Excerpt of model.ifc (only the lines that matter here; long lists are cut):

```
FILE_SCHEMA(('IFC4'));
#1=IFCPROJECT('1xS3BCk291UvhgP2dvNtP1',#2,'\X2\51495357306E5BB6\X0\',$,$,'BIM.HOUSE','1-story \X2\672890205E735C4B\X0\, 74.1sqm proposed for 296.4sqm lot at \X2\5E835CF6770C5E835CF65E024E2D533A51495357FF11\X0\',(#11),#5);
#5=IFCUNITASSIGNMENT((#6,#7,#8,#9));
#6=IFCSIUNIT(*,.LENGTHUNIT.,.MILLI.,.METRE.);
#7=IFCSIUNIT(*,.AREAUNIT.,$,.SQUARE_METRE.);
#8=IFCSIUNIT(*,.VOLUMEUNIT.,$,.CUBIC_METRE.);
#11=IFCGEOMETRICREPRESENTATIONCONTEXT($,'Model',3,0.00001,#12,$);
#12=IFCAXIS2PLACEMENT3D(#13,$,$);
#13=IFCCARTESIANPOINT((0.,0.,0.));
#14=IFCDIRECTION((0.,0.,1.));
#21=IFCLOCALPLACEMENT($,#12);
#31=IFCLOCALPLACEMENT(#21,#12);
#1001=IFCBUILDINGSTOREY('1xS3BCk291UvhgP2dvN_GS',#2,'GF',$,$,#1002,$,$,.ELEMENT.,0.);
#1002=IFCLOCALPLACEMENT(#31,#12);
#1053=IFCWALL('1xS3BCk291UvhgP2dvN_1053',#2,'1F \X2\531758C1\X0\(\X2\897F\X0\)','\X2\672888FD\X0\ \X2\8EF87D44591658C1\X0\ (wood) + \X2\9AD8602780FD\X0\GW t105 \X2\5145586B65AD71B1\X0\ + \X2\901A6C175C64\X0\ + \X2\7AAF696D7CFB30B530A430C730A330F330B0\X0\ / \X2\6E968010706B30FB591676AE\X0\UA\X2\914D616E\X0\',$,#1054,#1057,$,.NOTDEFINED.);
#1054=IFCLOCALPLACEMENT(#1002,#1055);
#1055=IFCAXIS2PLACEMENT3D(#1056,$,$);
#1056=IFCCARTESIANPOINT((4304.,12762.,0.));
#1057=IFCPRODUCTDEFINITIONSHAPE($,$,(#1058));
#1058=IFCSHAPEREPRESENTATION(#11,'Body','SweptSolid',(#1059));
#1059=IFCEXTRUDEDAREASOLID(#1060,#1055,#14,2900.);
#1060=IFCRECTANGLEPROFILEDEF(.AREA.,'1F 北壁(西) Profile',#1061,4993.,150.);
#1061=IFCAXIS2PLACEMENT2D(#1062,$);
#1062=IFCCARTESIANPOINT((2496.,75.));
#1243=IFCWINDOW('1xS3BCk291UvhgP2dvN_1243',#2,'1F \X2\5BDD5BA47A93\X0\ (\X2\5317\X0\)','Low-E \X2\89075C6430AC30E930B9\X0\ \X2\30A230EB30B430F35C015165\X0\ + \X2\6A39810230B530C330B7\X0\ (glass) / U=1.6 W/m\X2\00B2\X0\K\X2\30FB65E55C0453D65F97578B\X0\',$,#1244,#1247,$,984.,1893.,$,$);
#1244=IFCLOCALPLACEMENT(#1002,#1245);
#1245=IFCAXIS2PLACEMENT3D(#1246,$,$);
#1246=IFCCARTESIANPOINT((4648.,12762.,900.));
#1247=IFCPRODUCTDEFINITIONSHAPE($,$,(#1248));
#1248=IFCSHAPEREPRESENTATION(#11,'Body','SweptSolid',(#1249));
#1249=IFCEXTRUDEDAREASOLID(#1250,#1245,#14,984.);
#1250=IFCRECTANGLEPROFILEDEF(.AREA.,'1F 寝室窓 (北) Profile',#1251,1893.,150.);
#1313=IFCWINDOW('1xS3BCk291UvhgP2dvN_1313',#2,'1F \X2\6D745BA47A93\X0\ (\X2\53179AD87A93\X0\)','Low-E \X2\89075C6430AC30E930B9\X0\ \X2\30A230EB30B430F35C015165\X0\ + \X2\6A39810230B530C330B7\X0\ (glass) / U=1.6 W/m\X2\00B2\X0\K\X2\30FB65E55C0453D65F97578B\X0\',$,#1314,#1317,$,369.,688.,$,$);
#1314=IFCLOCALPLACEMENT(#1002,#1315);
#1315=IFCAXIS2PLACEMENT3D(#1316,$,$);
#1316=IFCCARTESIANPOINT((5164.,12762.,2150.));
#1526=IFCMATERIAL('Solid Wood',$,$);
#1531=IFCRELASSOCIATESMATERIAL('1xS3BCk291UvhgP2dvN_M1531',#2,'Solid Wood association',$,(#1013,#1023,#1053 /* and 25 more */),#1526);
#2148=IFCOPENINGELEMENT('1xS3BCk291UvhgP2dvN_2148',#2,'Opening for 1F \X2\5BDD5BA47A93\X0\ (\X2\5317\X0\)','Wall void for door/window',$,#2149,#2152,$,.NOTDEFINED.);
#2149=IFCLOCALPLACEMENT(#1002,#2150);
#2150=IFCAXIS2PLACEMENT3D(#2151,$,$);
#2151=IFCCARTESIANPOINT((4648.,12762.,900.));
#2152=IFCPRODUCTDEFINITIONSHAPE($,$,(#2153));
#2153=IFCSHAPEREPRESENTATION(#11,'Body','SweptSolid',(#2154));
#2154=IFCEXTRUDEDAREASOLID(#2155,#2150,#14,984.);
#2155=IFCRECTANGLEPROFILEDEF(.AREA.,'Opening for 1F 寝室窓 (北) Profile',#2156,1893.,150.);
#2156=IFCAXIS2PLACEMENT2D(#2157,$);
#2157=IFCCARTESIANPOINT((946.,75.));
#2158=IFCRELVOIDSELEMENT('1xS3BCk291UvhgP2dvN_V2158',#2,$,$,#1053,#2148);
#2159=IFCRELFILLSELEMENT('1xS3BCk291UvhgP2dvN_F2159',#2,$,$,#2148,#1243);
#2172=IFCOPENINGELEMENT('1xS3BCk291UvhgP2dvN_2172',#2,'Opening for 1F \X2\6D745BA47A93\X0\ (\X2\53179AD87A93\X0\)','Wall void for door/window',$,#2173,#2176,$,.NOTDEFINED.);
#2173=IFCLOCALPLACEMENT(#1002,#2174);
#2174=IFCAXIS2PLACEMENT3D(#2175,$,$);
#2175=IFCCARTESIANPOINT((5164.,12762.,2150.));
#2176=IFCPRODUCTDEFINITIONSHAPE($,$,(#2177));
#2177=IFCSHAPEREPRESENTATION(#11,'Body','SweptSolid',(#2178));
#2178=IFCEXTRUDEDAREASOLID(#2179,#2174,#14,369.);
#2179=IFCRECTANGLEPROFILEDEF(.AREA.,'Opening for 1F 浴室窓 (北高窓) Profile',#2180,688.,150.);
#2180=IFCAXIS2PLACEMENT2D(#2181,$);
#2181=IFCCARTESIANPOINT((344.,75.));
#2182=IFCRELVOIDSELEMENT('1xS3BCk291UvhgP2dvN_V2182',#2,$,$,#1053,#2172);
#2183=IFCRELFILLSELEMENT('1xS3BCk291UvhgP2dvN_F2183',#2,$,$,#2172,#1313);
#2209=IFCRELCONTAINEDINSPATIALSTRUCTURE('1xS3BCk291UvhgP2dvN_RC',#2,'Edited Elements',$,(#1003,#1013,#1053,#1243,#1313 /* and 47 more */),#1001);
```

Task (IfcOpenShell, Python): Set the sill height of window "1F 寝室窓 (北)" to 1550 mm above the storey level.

```python
import numpy as np
import ifcopenshell
import ifcopenshell.api.geometry
import ifcopenshell.geom
import ifcopenshell.util.element
import ifcopenshell.util.placement
import ifcopenshell.util.shape
import ifcopenshell.util.unit

model = ifcopenshell.open("model.ifc")
unit_scale = ifcopenshell.util.unit.calculate_unit_scale(model)

window = model.by_id(1243)
opening = window.FillsVoids[0].RelatingOpeningElement
storey = ifcopenshell.util.element.get_container(window, ifc_class="IfcBuildingStorey")
level = ifcopenshell.util.placement.get_local_placement(storey.ObjectPlacement)[2, 3]

# The opening's origin need not be at the sill, so measure its lowest point.
shape = ifcopenshell.geom.create_shape(ifcopenshell.geom.settings(), opening)
bottom = ifcopenshell.util.shape.get_shape_bottom_elevation(shape, shape.geometry) / unit_scale
dz = level + 1.55 / unit_scale - bottom

shift = np.array([0.0, 0.0, dz])
# The window is not placed relative to its opening, so move both.
for product in (opening, window):
    matrix = ifcopenshell.util.placement.get_local_placement(product.ObjectPlacement)
    matrix[:3, 3] += shift
    ifcopenshell.api.geometry.edit_object_placement(model, product=product, matrix=matrix, is_si=False)

print(f"moved by {dz * unit_scale:+.3f} m")

model.write("model_v2.ifc")
```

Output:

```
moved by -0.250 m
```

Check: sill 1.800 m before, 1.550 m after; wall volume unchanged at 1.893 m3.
